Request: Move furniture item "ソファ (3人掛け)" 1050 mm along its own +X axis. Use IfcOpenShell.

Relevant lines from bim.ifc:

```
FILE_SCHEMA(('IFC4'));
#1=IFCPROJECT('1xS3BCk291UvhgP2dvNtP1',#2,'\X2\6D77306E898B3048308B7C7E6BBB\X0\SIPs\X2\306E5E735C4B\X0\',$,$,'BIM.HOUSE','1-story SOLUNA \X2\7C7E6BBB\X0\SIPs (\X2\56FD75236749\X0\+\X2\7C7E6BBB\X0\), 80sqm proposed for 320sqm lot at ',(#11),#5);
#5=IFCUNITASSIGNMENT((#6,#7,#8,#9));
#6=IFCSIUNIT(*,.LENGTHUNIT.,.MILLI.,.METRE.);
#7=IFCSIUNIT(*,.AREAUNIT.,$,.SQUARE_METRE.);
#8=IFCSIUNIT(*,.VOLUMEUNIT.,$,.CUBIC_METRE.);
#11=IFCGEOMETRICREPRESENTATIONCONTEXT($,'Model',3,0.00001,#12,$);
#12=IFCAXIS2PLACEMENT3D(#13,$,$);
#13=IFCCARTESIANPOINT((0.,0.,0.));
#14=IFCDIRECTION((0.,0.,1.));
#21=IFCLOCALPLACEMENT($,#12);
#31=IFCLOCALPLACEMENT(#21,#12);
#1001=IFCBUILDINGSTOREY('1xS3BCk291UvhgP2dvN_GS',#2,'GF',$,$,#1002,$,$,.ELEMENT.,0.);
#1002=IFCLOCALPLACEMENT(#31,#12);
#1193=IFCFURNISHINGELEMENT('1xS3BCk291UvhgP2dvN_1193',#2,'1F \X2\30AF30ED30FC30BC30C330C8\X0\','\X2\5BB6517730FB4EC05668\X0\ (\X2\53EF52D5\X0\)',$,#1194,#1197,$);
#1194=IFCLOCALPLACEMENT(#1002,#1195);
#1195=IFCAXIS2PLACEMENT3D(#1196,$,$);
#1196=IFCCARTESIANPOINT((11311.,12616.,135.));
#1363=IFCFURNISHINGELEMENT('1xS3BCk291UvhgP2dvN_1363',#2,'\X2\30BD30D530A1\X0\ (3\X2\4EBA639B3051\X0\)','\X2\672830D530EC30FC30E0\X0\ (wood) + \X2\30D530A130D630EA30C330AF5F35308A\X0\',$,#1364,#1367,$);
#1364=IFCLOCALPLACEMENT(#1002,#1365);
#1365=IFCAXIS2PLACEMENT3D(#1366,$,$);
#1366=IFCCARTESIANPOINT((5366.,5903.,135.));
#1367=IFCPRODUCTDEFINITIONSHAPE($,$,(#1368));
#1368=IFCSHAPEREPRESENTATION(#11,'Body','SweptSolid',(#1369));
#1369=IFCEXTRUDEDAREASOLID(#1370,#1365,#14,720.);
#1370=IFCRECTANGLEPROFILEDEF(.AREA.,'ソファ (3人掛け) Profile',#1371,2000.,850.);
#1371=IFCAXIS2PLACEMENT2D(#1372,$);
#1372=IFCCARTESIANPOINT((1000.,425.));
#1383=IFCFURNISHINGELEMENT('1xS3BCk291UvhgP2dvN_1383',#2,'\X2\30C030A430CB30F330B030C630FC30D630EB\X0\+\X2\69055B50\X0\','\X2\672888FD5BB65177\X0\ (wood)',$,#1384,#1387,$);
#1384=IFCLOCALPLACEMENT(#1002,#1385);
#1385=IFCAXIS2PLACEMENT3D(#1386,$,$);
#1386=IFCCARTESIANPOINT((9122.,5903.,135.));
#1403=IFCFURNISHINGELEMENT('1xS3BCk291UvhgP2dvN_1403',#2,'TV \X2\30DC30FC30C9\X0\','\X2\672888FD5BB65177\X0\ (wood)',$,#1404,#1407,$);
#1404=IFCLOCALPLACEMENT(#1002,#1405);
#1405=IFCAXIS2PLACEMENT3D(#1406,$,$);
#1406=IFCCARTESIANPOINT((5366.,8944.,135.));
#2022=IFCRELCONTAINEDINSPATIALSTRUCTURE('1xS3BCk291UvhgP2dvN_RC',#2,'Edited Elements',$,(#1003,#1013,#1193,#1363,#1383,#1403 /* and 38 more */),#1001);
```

```python
import ifcopenshell
import ifcopenshell.api.geometry
import ifcopenshell.util.placement

model = ifcopenshell.open("bim.ifc")

item = model.by_guid("1xS3BCk291UvhgP2dvN_1363")
matrix = ifcopenshell.util.placement.get_local_placement(item.ObjectPlacement)
matrix[:3, 3] += matrix[:3, 0] * 1050.0
ifcopenshell.api.geometry.edit_object_placement(model, product=item, matrix=matrix, is_si=False)

print(ifcopenshell.util.placement.get_local_placement(item.ObjectPlacement).round(3) + 0.0)

model.write("bim-out.ifc")
```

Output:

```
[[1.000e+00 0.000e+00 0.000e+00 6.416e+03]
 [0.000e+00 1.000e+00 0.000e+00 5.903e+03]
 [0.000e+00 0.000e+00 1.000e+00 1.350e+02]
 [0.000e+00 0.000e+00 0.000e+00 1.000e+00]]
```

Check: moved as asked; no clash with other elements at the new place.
